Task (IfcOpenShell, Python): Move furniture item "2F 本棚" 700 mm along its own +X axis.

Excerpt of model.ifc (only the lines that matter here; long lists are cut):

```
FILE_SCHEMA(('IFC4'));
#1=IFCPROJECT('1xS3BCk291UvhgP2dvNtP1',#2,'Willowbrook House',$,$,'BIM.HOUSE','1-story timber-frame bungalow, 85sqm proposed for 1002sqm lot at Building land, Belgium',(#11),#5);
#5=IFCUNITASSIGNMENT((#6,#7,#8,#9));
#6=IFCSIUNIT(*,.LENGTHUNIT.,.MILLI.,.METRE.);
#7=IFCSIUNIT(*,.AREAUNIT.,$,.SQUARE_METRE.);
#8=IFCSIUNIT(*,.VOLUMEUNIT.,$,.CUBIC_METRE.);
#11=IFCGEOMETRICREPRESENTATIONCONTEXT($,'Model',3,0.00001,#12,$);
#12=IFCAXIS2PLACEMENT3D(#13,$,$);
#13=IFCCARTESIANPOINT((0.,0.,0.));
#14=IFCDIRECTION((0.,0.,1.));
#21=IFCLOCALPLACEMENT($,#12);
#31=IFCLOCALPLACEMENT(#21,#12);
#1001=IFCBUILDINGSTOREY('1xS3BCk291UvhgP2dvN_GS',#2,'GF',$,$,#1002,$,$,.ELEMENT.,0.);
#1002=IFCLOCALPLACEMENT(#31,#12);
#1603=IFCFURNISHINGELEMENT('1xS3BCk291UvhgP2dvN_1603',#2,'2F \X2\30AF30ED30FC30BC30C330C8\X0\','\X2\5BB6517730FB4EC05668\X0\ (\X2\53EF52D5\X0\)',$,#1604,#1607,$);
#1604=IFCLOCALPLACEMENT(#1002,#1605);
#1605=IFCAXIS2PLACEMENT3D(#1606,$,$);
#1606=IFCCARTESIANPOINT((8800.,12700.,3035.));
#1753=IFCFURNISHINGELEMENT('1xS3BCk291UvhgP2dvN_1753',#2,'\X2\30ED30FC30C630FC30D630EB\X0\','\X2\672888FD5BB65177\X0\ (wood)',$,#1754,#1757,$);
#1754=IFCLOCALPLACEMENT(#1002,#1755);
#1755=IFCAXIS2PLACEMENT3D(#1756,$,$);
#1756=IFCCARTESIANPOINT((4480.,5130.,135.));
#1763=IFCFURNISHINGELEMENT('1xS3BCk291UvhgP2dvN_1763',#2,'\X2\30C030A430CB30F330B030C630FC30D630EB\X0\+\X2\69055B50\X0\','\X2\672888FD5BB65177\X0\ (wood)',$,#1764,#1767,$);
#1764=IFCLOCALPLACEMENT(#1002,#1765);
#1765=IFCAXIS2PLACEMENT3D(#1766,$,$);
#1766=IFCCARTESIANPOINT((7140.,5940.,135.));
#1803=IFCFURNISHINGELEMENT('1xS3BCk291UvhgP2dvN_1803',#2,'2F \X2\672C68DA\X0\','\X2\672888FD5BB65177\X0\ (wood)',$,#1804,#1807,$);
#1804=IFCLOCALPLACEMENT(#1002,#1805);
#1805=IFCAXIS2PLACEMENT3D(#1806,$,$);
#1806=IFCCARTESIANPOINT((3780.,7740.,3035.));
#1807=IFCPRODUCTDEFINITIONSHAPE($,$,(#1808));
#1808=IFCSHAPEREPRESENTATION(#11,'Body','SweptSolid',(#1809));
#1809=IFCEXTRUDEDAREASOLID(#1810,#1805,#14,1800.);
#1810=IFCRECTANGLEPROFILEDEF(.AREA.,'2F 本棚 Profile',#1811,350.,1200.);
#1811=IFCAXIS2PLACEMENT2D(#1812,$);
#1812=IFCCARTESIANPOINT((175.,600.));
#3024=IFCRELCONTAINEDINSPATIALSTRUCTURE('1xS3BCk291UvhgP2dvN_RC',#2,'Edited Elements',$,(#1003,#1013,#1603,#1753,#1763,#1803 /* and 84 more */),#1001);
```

```python
import ifcopenshell
import ifcopenshell.api.geometry
import ifcopenshell.util.placement

model = ifcopenshell.open("model.ifc")

item = model.by_guid("1xS3BCk291UvhgP2dvN_1803")
matrix = ifcopenshell.util.placement.get_local_placement(item.ObjectPlacement)
matrix[:3, 3] += matrix[:3, 0] * 700.0
ifcopenshell.api.geometry.edit_object_placement(model, product=item, matrix=matrix, is_si=False)

print(ifcopenshell.util.placement.get_local_placement(item.ObjectPlacement).round(3) + 0.0)

model.write("model-out.ifc")
```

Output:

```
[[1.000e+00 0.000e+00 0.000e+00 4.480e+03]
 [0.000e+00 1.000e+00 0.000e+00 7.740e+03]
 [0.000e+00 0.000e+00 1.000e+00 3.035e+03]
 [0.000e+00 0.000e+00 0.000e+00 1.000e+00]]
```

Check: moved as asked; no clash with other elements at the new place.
